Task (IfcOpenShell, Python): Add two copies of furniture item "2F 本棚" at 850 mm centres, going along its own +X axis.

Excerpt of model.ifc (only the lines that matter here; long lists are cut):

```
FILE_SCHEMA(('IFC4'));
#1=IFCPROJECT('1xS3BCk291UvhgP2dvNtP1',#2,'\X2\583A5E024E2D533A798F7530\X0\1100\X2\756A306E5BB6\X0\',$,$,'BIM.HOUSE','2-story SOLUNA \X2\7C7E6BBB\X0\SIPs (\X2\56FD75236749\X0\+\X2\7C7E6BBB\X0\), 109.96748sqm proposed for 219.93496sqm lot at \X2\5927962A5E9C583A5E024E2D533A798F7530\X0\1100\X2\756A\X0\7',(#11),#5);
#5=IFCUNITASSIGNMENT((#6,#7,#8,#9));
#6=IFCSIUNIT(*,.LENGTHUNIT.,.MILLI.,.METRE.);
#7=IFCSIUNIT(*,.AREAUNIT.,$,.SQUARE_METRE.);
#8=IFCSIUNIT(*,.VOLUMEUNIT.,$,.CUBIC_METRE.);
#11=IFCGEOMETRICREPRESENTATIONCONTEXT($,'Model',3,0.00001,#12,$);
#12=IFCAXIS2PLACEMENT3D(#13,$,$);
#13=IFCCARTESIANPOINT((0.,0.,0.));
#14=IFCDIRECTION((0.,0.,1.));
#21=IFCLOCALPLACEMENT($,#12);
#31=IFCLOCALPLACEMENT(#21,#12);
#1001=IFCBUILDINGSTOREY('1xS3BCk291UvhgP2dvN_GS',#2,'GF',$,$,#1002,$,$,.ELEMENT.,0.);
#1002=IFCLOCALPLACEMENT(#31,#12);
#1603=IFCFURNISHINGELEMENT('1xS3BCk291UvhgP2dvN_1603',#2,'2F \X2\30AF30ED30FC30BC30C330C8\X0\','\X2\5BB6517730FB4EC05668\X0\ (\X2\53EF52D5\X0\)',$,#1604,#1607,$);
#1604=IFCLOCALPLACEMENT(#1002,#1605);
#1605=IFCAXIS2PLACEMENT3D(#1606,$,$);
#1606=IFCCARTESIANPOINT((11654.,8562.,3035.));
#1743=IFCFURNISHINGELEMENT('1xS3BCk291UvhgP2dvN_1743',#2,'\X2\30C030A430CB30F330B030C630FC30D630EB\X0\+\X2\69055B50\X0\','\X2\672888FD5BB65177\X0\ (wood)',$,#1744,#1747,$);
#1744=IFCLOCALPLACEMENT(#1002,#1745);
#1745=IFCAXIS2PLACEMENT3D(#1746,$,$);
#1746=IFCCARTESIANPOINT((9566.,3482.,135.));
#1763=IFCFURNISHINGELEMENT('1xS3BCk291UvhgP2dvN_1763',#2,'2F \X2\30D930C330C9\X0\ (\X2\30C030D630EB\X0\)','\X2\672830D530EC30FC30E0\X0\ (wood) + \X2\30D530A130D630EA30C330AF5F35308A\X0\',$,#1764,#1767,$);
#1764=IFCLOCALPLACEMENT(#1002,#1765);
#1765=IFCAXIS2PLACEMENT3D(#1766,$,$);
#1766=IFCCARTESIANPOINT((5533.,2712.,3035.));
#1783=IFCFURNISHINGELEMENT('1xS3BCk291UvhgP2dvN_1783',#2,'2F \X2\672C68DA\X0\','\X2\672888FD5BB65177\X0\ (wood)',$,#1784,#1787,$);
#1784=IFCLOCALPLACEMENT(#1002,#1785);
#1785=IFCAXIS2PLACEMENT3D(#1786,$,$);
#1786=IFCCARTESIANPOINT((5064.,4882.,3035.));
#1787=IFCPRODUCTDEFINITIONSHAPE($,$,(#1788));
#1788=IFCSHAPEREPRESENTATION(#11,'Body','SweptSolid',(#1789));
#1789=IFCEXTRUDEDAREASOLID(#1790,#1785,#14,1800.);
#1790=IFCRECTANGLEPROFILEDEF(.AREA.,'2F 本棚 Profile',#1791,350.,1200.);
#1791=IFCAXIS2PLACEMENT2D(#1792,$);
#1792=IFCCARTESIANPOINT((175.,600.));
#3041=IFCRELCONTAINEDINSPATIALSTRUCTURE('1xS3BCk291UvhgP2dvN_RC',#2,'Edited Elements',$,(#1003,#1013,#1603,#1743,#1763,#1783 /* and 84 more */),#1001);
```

```python
import ifcopenshell
import ifcopenshell.api.geometry
import ifcopenshell.api.root
import ifcopenshell.util.element
import ifcopenshell.util.placement
import ifcopenshell.util.unit

model = ifcopenshell.open("model.ifc")
unit_scale = ifcopenshell.util.unit.calculate_unit_scale(model)


def reuse_history(source, copy):
    """copy_class also copies each property set's owner history, people and application; keep the originals."""
    for rel in copy.IsDefinedBy:
        if rel.is_a("IfcRelDefinesByProperties") and (history := rel.RelatingPropertyDefinition.OwnerHistory):
            rel.RelatingPropertyDefinition.OwnerHistory = source.OwnerHistory
            ifcopenshell.util.element.remove_deep2(model, history)


source = model.by_guid("1xS3BCk291UvhgP2dvN_1783")
base = ifcopenshell.util.placement.get_local_placement(source.ObjectPlacement)
step = base[:3, 0] * 0.85 / unit_scale

for i in range(1, 3):
    copy = ifcopenshell.api.root.copy_class(model, product=source)
    copy.Representation = ifcopenshell.util.element.copy_deep(
        model, source.Representation, exclude=["IfcGeometricRepresentationContext", "IfcRepresentationMap"]
    )
    reuse_history(source, copy)
    matrix = base.copy()
    matrix[:3, 3] += i * step
    print("added at", matrix[:3, 3].round(3) + 0.0)
    ifcopenshell.api.geometry.edit_object_placement(model, product=copy, matrix=matrix, is_si=False)

model.write("model_rev.ifc")
```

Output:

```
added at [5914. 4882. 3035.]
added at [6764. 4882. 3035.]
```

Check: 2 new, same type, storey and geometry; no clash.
